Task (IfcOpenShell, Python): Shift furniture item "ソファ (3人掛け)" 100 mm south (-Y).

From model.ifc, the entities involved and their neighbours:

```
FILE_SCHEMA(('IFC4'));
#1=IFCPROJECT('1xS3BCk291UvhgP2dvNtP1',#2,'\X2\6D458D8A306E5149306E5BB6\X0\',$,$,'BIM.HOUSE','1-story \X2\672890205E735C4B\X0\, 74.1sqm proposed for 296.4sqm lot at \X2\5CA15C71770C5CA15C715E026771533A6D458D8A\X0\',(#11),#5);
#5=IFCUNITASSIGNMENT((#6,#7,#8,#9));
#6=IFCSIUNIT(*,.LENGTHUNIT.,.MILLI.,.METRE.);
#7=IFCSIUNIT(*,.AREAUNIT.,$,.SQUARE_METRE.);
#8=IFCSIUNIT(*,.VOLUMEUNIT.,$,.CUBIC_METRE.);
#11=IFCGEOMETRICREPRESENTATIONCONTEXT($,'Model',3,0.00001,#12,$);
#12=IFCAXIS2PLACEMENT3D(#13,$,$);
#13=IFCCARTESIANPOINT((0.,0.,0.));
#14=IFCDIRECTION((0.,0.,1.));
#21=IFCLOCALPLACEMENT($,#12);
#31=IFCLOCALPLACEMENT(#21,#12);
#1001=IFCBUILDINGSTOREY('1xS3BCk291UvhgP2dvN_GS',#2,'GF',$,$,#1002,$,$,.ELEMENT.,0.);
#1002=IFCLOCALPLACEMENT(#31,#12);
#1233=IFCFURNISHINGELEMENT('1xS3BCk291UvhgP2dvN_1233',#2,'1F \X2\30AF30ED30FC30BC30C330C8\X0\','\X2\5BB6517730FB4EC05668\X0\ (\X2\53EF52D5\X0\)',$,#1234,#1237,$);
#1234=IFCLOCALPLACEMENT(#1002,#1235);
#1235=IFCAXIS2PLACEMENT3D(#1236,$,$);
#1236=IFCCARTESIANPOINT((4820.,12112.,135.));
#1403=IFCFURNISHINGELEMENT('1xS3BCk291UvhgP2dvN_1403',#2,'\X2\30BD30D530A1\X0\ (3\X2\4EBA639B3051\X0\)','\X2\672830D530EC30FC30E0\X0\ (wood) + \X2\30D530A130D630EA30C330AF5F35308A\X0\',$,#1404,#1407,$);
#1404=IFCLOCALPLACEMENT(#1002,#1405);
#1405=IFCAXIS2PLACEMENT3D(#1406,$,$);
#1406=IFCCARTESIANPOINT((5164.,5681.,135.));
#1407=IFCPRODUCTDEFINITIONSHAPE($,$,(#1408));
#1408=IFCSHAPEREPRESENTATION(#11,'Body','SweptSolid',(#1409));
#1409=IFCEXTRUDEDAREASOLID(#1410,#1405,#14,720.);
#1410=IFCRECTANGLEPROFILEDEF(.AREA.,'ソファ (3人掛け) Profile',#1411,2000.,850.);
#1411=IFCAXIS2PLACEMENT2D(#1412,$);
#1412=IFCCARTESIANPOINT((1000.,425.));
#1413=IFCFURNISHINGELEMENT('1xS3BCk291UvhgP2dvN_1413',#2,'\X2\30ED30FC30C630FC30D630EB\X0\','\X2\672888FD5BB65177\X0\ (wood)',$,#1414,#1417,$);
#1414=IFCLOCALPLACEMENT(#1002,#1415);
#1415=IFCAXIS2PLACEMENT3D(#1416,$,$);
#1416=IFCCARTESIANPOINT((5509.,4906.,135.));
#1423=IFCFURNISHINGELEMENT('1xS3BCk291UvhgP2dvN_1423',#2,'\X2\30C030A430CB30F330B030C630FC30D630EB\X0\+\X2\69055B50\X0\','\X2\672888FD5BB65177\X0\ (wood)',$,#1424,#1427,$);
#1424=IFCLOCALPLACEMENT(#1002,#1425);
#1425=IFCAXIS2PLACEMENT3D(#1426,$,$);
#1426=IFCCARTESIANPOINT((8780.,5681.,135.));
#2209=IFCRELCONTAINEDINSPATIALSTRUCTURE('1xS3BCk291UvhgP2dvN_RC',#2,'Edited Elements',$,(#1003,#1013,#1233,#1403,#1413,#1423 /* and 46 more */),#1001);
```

```python
import ifcopenshell
import ifcopenshell.api.geometry
import ifcopenshell.util.placement
import ifcopenshell.util.unit

model = ifcopenshell.open("model.ifc")
unit_scale = ifcopenshell.util.unit.calculate_unit_scale(model)

item = model.by_guid("1xS3BCk291UvhgP2dvN_1403")
matrix = ifcopenshell.util.placement.get_local_placement(item.ObjectPlacement)
matrix[1, 3] -= 0.1 / unit_scale
ifcopenshell.api.geometry.edit_object_placement(model, product=item, matrix=matrix, is_si=False)

print(ifcopenshell.util.placement.get_local_placement(item.ObjectPlacement).round(3) + 0.0)

model.write("model_edited.ifc")
```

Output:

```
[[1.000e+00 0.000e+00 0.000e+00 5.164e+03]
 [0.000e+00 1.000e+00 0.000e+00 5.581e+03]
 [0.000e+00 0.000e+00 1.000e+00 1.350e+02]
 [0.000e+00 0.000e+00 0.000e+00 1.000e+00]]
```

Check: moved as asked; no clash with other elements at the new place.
